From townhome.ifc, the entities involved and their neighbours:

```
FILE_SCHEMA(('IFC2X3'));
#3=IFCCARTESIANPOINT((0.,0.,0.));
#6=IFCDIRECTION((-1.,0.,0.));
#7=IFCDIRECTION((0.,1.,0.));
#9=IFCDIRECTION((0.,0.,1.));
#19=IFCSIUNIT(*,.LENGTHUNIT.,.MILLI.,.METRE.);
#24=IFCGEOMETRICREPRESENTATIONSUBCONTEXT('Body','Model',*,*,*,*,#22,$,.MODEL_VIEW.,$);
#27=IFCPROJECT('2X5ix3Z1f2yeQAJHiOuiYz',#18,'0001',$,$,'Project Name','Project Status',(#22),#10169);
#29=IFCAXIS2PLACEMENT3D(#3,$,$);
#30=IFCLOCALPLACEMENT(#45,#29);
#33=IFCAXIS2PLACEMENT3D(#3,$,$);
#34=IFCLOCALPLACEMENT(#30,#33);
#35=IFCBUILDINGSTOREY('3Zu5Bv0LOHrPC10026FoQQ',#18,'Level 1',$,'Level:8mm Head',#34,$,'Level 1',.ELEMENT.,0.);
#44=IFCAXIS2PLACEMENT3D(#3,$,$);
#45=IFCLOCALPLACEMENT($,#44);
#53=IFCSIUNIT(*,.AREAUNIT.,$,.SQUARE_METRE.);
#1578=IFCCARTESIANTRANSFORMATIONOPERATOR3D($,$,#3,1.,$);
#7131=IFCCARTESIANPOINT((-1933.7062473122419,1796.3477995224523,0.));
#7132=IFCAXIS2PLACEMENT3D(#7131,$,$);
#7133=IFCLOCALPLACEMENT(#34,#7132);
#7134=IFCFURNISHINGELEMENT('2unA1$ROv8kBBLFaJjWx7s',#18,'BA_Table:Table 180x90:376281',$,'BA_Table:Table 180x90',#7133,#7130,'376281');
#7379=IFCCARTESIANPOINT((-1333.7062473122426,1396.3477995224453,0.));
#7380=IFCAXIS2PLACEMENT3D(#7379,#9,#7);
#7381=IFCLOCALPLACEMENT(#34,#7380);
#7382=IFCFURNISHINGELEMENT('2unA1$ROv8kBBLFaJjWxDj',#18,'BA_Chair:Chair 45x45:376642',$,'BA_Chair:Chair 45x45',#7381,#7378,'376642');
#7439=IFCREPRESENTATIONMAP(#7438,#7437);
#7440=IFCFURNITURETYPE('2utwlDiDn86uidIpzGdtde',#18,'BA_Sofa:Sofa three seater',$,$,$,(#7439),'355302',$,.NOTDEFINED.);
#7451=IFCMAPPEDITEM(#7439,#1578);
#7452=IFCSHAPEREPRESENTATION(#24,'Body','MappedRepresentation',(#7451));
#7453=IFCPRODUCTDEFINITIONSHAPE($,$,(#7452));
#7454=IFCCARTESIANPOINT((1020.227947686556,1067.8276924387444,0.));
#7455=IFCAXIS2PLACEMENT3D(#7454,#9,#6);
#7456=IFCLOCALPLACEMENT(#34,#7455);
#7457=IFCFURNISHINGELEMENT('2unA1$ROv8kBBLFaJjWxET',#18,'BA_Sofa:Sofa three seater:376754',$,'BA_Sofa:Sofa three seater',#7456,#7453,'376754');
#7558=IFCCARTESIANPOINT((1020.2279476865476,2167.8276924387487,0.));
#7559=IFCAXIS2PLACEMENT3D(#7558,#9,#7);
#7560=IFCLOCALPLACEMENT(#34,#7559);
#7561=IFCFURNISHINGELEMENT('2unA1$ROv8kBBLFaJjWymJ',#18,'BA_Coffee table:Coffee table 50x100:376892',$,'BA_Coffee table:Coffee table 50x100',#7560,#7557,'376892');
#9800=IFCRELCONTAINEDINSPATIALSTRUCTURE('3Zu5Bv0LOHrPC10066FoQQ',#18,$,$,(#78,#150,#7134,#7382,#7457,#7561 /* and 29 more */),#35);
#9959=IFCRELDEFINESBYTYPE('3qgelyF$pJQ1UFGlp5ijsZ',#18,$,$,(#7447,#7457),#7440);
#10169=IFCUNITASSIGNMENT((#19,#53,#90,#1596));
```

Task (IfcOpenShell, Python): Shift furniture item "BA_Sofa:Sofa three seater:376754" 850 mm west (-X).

```python
import ifcopenshell
import ifcopenshell.api.geometry
import ifcopenshell.util.placement
import ifcopenshell.util.unit

model = ifcopenshell.open("townhome.ifc")
unit_scale = ifcopenshell.util.unit.calculate_unit_scale(model)

item = model.by_id(7457)
matrix = ifcopenshell.util.placement.get_local_placement(item.ObjectPlacement)
matrix[0, 3] -= 0.85 / unit_scale
ifcopenshell.api.geometry.edit_object_placement(model, product=item, matrix=matrix, is_si=False)

print(ifcopenshell.util.placement.get_local_placement(item.ObjectPlacement).round(3) + 0.0)

model.write("townhome_v2.ifc")
```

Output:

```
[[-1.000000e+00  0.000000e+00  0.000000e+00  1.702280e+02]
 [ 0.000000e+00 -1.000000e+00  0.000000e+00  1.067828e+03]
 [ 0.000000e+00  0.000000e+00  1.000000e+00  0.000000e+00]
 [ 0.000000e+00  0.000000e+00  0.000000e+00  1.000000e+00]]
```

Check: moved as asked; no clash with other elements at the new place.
